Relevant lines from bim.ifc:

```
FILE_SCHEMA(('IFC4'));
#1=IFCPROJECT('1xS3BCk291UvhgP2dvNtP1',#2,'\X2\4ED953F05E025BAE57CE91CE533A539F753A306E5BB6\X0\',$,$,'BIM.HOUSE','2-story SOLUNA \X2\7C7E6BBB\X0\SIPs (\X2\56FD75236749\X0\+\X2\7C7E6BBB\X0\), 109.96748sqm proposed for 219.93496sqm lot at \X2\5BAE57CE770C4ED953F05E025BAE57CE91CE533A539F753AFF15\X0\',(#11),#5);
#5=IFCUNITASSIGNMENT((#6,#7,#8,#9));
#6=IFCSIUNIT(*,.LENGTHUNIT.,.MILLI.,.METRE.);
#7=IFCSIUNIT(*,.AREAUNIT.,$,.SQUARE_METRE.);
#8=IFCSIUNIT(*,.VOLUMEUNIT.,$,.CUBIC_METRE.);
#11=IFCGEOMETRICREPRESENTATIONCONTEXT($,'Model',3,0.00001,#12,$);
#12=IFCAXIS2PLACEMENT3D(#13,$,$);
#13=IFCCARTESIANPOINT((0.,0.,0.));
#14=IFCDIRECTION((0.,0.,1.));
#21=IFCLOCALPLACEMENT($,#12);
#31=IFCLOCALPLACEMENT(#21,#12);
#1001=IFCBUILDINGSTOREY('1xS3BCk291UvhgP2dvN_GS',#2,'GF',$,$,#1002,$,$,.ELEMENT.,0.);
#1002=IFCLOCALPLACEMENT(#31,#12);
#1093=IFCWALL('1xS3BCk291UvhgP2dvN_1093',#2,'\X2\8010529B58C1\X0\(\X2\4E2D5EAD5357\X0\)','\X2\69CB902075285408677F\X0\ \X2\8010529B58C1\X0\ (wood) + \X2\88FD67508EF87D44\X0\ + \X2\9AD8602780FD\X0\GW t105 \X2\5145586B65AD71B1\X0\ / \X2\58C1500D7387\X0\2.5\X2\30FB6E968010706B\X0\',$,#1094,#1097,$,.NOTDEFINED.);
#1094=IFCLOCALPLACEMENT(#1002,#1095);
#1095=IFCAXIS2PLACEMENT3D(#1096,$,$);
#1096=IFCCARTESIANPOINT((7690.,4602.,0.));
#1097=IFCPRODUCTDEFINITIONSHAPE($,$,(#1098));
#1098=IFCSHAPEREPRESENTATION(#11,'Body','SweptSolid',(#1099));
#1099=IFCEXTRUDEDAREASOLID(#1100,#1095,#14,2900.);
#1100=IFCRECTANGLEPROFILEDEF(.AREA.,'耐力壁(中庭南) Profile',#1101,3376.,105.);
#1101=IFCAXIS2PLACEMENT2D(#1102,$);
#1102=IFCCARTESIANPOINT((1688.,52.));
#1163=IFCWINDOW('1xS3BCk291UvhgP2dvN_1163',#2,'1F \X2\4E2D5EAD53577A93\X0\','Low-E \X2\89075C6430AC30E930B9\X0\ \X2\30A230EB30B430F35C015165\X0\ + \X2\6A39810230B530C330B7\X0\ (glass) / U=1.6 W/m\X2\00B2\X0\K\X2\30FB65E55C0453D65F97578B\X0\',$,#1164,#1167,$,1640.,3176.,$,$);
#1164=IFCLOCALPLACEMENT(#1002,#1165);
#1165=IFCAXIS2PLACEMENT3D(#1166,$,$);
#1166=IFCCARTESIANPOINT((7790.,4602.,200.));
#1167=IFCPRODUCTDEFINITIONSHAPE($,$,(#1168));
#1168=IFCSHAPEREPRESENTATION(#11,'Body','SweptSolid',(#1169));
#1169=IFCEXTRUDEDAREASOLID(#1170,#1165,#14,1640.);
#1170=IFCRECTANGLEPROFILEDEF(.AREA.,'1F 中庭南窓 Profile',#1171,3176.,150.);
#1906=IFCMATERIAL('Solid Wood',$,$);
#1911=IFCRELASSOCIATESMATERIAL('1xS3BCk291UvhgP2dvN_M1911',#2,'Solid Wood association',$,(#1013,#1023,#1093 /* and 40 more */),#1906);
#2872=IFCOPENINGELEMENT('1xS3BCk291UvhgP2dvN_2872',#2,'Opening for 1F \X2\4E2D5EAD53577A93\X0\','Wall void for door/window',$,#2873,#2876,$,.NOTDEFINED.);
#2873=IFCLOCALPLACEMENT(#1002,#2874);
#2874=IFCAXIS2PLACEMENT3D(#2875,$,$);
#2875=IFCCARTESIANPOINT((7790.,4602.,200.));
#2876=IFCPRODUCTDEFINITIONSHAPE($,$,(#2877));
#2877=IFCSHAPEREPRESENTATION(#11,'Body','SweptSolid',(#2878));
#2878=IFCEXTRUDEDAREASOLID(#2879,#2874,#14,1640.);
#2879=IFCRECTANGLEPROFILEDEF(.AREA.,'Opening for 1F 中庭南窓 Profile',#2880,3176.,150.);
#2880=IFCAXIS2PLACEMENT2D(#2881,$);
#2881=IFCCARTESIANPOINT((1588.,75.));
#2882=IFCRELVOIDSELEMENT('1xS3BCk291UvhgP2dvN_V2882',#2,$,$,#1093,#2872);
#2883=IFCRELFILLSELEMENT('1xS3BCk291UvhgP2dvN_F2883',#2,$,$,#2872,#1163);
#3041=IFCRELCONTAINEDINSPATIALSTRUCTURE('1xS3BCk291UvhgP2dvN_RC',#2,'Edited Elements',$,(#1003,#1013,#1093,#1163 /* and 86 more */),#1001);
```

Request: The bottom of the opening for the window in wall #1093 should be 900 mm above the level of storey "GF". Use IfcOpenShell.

```python
import numpy as np
import ifcopenshell
import ifcopenshell.api.geometry
import ifcopenshell.geom
import ifcopenshell.util.element
import ifcopenshell.util.placement
import ifcopenshell.util.shape
import ifcopenshell.util.unit

model = ifcopenshell.open("bim.ifc")
unit_scale = ifcopenshell.util.unit.calculate_unit_scale(model)

window = model.by_id(1163)
opening = window.FillsVoids[0].RelatingOpeningElement
storey = ifcopenshell.util.element.get_container(window, ifc_class="IfcBuildingStorey")
level = ifcopenshell.util.placement.get_local_placement(storey.ObjectPlacement)[2, 3]

# The opening's origin need not be at the sill, so measure its lowest point.
shape = ifcopenshell.geom.create_shape(ifcopenshell.geom.settings(), opening)
bottom = ifcopenshell.util.shape.get_shape_bottom_elevation(shape, shape.geometry) / unit_scale
dz = level + 0.9 / unit_scale - bottom

shift = np.array([0.0, 0.0, dz])
# The window is not placed relative to its opening, so move both.
for product in (opening, window):
    matrix = ifcopenshell.util.placement.get_local_placement(product.ObjectPlacement)
    matrix[:3, 3] += shift
    ifcopenshell.api.geometry.edit_object_placement(model, product=product, matrix=matrix, is_si=False)

print(f"moved by {dz * unit_scale:+.3f} m")

model.write("bim_updated.ifc")
```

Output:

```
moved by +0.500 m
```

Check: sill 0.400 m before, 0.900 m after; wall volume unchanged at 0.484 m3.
